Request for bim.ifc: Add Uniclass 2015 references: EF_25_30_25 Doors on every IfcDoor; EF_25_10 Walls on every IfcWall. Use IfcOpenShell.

First a look at what the model holds.

```python
import ifcopenshell

model = ifcopenshell.open("bim.ifc")
print(model.schema)
print("classifications:", [c.Name for c in model.by_type("IfcClassification")])
for ifc_class in ("IfcDoor", "IfcRoof", "IfcStair", "IfcWall", "IfcWindow"):
    print(ifc_class, len(model.by_type(ifc_class)))
```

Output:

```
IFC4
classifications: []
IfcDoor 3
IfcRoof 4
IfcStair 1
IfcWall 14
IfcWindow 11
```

```python
import ifcopenshell
import ifcopenshell.api.classification

model = ifcopenshell.open("bim.ifc")

system = ifcopenshell.api.classification.add_classification(model, classification="Uniclass 2015")

codes = {
    "IfcDoor": ("EF_25_30_25", "Doors"),
    "IfcWall": ("EF_25_10", "Walls"),
}
for ifc_class, (code, name) in codes.items():
    products = model.by_type(ifc_class)
    ifcopenshell.api.classification.add_reference(
        model, products=products, classification=system, identification=code, name=name
    )
    print(code, len(products))

model.write("bim_rev.ifc")
```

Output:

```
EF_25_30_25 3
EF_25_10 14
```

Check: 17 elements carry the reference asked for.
